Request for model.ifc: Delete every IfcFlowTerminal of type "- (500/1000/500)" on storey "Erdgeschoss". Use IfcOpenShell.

First a look at what the model holds.

```python
import ifcopenshell
import ifcopenshell.util.element

model = ifcopenshell.open("model.ifc")
print(model.schema)
storey = next(s for s in model.by_type("IfcBuildingStorey") if s.Name == "Erdgeschoss")
terminals = [e for e in ifcopenshell.util.element.get_decomposition(storey) if e.is_a("IfcFlowTerminal")]
seen = {}
for e in terminals:
    element_type = ifcopenshell.util.element.get_type(e)
    name = element_type.Name if element_type not in (None, e) else None
    seen[name] = seen.get(name, 0) + 1
for name, count in sorted(seen.items(), key=str):
    print(count, "x", name)
```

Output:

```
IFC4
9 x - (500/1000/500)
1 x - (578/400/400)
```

```python
import ifcopenshell
import ifcopenshell.api.root
import ifcopenshell.util.element

model = ifcopenshell.open("model.ifc")

storey = next(s for s in model.by_type("IfcBuildingStorey") if s.Name == "Erdgeschoss")
terminals = [e for e in ifcopenshell.util.element.get_decomposition(storey) if e.is_a("IfcFlowTerminal")]
targets = [e for e in terminals if (t := ifcopenshell.util.element.get_type(e)) not in (None, e) and t.Name == "- (500/1000/500)"]

for e in targets:
    ifcopenshell.api.root.remove_product(model, product=e)
print(len(targets), "removed")

model.write("model_updated.ifc")
```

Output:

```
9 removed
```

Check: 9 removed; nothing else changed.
